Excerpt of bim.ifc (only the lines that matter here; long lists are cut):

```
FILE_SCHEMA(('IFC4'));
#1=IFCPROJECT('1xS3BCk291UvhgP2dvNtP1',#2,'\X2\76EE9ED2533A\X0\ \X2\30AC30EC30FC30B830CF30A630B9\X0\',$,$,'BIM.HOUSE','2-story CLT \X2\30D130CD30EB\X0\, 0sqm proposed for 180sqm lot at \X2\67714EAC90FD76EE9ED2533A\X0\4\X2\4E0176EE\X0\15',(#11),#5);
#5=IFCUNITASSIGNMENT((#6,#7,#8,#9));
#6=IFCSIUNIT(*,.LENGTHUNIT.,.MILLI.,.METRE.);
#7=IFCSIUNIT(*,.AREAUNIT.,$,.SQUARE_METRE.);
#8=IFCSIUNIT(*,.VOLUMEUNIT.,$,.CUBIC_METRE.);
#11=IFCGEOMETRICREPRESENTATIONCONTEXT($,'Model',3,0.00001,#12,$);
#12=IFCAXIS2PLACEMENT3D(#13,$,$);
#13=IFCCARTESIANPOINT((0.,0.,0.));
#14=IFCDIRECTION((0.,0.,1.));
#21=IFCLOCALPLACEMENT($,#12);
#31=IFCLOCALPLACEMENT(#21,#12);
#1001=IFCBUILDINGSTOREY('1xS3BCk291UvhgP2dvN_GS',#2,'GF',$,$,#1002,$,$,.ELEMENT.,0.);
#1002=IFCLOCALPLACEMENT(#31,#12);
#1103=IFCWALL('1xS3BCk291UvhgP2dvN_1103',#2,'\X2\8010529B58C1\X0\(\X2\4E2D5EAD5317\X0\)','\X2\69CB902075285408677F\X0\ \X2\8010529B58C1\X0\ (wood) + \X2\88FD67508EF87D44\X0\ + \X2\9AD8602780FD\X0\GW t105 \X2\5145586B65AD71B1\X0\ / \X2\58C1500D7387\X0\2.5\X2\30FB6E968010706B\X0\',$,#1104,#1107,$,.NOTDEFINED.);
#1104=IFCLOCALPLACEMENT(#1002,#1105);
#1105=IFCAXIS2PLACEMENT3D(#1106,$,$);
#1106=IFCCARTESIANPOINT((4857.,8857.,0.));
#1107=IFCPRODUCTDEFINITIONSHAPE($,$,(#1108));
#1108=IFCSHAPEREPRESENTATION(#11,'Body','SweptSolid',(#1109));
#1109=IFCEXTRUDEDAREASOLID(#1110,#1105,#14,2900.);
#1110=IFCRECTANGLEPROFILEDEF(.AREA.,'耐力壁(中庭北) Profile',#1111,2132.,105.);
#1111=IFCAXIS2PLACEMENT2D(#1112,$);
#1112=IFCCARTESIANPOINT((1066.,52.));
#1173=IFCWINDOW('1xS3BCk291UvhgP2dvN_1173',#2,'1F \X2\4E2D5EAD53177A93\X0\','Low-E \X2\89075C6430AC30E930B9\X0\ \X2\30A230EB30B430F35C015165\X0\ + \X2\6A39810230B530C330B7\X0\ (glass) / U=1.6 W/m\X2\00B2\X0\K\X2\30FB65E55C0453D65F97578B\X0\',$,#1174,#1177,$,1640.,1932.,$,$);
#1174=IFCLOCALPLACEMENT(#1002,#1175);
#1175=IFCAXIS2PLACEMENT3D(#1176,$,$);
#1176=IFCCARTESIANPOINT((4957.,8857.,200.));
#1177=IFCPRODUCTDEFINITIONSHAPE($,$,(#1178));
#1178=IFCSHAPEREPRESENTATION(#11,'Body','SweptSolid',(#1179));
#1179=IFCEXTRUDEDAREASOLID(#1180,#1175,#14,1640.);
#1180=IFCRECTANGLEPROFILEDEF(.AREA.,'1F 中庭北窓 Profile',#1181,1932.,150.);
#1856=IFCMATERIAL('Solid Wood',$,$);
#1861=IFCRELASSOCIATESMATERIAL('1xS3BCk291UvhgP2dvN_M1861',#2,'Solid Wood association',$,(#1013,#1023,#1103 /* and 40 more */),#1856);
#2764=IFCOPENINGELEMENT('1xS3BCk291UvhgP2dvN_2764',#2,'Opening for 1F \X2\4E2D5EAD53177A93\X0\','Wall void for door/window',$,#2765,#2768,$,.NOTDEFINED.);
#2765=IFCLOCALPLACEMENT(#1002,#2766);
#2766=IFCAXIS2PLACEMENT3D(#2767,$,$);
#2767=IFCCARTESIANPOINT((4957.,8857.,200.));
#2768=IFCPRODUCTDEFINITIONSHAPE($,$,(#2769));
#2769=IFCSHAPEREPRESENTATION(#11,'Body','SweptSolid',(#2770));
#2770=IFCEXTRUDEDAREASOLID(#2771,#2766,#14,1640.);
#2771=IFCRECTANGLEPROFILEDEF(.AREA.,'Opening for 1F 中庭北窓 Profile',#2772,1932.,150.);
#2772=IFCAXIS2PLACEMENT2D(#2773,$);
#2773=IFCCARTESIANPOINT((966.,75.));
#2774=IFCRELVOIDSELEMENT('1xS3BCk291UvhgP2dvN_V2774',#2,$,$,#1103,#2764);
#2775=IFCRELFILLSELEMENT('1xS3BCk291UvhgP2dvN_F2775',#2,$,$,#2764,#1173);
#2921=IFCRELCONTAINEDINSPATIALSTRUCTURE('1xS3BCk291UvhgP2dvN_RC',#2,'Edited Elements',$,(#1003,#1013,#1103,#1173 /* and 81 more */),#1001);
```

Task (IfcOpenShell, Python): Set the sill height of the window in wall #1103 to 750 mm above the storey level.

```python
import numpy as np
import ifcopenshell
import ifcopenshell.api.geometry
import ifcopenshell.geom
import ifcopenshell.util.element
import ifcopenshell.util.placement
import ifcopenshell.util.shape
import ifcopenshell.util.unit

model = ifcopenshell.open("bim.ifc")
unit_scale = ifcopenshell.util.unit.calculate_unit_scale(model)

window = model.by_guid("1xS3BCk291UvhgP2dvN_1173")
opening = window.FillsVoids[0].RelatingOpeningElement
storey = ifcopenshell.util.element.get_container(window, ifc_class="IfcBuildingStorey")
level = ifcopenshell.util.placement.get_local_placement(storey.ObjectPlacement)[2, 3]

# The opening's origin need not be at the sill, so measure its lowest point.
shape = ifcopenshell.geom.create_shape(ifcopenshell.geom.settings(), opening)
bottom = ifcopenshell.util.shape.get_shape_bottom_elevation(shape, shape.geometry) / unit_scale
dz = level + 0.75 / unit_scale - bottom

shift = np.array([0.0, 0.0, dz])
# The window is not placed relative to its opening, so move both.
for product in (opening, window):
    matrix = ifcopenshell.util.placement.get_local_placement(product.ObjectPlacement)
    matrix[:3, 3] += shift
    ifcopenshell.api.geometry.edit_object_placement(model, product=product, matrix=matrix, is_si=False)

print(f"moved by {dz * unit_scale:+.3f} m")

model.write("bim_rev.ifc")
```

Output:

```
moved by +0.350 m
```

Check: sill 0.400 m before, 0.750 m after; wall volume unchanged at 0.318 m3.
